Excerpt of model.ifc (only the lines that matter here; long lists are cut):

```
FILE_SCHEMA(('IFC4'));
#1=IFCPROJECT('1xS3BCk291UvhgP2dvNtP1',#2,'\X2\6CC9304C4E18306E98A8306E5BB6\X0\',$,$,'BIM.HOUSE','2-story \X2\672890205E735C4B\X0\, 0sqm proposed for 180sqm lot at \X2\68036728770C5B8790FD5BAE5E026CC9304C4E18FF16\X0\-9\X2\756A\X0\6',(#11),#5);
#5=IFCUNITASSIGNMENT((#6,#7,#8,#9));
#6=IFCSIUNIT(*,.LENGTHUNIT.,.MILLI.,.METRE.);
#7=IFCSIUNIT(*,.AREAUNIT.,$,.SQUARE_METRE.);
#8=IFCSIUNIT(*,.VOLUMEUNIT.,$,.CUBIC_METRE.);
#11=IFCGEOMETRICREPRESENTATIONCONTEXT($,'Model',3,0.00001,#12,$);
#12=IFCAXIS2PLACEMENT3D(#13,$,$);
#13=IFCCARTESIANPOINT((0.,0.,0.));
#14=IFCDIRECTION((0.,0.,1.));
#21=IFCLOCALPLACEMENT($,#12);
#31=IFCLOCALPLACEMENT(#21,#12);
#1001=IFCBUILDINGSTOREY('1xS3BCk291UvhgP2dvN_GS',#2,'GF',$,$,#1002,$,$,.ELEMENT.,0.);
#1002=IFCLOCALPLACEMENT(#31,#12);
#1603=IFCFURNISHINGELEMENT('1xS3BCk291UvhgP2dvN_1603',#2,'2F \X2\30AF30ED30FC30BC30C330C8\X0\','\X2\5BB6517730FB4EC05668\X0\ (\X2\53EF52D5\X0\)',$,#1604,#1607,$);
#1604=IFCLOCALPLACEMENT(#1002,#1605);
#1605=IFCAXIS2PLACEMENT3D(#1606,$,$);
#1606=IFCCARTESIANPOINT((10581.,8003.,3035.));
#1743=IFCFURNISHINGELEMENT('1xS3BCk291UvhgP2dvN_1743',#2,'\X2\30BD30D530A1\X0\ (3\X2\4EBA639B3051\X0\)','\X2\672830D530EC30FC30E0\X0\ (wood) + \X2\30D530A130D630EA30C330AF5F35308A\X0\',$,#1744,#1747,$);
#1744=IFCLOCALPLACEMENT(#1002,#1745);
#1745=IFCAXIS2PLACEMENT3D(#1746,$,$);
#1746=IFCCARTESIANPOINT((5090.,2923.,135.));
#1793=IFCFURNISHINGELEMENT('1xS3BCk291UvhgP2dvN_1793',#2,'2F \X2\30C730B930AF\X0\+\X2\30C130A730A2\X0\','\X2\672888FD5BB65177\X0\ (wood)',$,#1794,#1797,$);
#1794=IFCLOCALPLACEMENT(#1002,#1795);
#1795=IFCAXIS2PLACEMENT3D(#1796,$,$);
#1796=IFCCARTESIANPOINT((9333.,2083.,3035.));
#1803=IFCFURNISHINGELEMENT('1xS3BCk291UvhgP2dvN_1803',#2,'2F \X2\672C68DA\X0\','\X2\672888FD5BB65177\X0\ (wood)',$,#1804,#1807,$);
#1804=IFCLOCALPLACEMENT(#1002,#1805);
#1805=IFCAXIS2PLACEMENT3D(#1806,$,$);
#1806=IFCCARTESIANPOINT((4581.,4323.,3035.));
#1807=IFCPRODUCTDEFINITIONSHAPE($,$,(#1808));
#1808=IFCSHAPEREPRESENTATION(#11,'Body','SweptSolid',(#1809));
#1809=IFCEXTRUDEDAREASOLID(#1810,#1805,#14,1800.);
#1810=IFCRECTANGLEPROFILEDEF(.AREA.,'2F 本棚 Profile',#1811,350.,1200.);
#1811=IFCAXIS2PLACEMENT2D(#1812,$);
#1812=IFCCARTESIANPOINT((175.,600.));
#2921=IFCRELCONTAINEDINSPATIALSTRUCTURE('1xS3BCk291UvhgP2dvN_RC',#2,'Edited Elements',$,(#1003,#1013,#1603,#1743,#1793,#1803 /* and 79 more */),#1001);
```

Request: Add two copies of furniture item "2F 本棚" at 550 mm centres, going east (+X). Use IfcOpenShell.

```python
import numpy as np
import ifcopenshell
import ifcopenshell.api.geometry
import ifcopenshell.api.root
import ifcopenshell.util.element
import ifcopenshell.util.placement
import ifcopenshell.util.unit

model = ifcopenshell.open("model.ifc")
unit_scale = ifcopenshell.util.unit.calculate_unit_scale(model)


def reuse_history(source, copy):
    """copy_class also copies each property set's owner history, people and application; keep the originals."""
    for rel in copy.IsDefinedBy:
        if rel.is_a("IfcRelDefinesByProperties") and (history := rel.RelatingPropertyDefinition.OwnerHistory):
            rel.RelatingPropertyDefinition.OwnerHistory = source.OwnerHistory
            ifcopenshell.util.element.remove_deep2(model, history)


source = model.by_guid("1xS3BCk291UvhgP2dvN_1803")
base = ifcopenshell.util.placement.get_local_placement(source.ObjectPlacement)
step = np.array([1.0, 0.0, 0.0]) * 0.55 / unit_scale

for i in range(1, 3):
    copy = ifcopenshell.api.root.copy_class(model, product=source)
    copy.Representation = ifcopenshell.util.element.copy_deep(
        model, source.Representation, exclude=["IfcGeometricRepresentationContext", "IfcRepresentationMap"]
    )
    reuse_history(source, copy)
    matrix = base.copy()
    matrix[:3, 3] += i * step
    print("added at", matrix[:3, 3].round(3) + 0.0)
    ifcopenshell.api.geometry.edit_object_placement(model, product=copy, matrix=matrix, is_si=False)

model.write("model-out.ifc")
```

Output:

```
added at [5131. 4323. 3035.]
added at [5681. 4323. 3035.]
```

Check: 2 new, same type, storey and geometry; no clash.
